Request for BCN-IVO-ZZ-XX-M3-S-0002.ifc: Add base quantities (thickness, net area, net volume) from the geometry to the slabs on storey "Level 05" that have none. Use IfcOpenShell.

First a look at what the model holds.

```python
import ifcopenshell
import ifcopenshell.util.element
import ifcopenshell.util.unit

model = ifcopenshell.open("BCN-IVO-ZZ-XX-M3-S-0002.ifc")
print(model.schema)
for unit_type in ("LENGTHUNIT", "AREAUNIT", "VOLUMEUNIT"):
    print(unit_type, ifcopenshell.util.unit.calculate_unit_scale(model, unit_type))
storey = next(s for s in model.by_type("IfcBuildingStorey") if s.Name == "Level 05")
slabs = [e for e in ifcopenshell.util.element.get_decomposition(storey) if e.is_a("IfcSlab")]
for e in sorted(slabs, key=lambda e: e.id()):
    print(e.id(), e.is_a(), e.Name, list(ifcopenshell.util.element.get_psets(e, qtos_only=True)), sep=" | ")
```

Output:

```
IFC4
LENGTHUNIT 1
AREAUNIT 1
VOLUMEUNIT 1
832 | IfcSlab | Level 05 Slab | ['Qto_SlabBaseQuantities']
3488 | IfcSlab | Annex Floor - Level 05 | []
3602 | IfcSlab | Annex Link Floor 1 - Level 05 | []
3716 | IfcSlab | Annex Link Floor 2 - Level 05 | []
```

```python
import ifcopenshell
import ifcopenshell.api.pset
import ifcopenshell.geom
import ifcopenshell.util.element
import ifcopenshell.util.shape
import ifcopenshell.util.unit

model = ifcopenshell.open("BCN-IVO-ZZ-XX-M3-S-0002.ifc")
unit_scale = ifcopenshell.util.unit.calculate_unit_scale(model)
area_scale = ifcopenshell.util.unit.calculate_unit_scale(model, "AREAUNIT")
volume_scale = ifcopenshell.util.unit.calculate_unit_scale(model, "VOLUMEUNIT")
settings = ifcopenshell.geom.settings()

storey = next(s for s in model.by_type("IfcBuildingStorey") if s.Name == "Level 05")
slabs = [e for e in ifcopenshell.util.element.get_decomposition(storey) if e.is_a("IfcSlab")]

for e in sorted(slabs, key=lambda e: e.id()):
    if ifcopenshell.util.element.get_psets(e, qtos_only=True, should_inherit=False):
        continue
    # Geometry comes back in metres, in the element's own axes.
    shape = ifcopenshell.geom.create_shape(settings, e)
    values = {
        "Width": ifcopenshell.util.shape.get_z(shape.geometry) / unit_scale,
        "NetArea": ifcopenshell.util.shape.get_footprint_area(shape.geometry) / area_scale,
        "NetVolume": ifcopenshell.util.shape.get_volume(shape.geometry) / volume_scale,
    }
    qto = ifcopenshell.api.pset.add_qto(model, product=e, name="Qto_SlabBaseQuantities")
    ifcopenshell.api.pset.edit_qto(model, qto=qto, properties=values)
    print(e.id(), {k: round(v, 3) for k, v in values.items()})

model.write("BCN-IVO-ZZ-XX-M3-S-0002_rev.ifc")
```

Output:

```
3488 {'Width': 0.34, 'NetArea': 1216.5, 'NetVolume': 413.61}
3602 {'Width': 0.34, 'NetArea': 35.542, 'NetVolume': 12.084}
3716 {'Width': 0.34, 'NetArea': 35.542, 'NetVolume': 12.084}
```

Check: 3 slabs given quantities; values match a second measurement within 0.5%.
